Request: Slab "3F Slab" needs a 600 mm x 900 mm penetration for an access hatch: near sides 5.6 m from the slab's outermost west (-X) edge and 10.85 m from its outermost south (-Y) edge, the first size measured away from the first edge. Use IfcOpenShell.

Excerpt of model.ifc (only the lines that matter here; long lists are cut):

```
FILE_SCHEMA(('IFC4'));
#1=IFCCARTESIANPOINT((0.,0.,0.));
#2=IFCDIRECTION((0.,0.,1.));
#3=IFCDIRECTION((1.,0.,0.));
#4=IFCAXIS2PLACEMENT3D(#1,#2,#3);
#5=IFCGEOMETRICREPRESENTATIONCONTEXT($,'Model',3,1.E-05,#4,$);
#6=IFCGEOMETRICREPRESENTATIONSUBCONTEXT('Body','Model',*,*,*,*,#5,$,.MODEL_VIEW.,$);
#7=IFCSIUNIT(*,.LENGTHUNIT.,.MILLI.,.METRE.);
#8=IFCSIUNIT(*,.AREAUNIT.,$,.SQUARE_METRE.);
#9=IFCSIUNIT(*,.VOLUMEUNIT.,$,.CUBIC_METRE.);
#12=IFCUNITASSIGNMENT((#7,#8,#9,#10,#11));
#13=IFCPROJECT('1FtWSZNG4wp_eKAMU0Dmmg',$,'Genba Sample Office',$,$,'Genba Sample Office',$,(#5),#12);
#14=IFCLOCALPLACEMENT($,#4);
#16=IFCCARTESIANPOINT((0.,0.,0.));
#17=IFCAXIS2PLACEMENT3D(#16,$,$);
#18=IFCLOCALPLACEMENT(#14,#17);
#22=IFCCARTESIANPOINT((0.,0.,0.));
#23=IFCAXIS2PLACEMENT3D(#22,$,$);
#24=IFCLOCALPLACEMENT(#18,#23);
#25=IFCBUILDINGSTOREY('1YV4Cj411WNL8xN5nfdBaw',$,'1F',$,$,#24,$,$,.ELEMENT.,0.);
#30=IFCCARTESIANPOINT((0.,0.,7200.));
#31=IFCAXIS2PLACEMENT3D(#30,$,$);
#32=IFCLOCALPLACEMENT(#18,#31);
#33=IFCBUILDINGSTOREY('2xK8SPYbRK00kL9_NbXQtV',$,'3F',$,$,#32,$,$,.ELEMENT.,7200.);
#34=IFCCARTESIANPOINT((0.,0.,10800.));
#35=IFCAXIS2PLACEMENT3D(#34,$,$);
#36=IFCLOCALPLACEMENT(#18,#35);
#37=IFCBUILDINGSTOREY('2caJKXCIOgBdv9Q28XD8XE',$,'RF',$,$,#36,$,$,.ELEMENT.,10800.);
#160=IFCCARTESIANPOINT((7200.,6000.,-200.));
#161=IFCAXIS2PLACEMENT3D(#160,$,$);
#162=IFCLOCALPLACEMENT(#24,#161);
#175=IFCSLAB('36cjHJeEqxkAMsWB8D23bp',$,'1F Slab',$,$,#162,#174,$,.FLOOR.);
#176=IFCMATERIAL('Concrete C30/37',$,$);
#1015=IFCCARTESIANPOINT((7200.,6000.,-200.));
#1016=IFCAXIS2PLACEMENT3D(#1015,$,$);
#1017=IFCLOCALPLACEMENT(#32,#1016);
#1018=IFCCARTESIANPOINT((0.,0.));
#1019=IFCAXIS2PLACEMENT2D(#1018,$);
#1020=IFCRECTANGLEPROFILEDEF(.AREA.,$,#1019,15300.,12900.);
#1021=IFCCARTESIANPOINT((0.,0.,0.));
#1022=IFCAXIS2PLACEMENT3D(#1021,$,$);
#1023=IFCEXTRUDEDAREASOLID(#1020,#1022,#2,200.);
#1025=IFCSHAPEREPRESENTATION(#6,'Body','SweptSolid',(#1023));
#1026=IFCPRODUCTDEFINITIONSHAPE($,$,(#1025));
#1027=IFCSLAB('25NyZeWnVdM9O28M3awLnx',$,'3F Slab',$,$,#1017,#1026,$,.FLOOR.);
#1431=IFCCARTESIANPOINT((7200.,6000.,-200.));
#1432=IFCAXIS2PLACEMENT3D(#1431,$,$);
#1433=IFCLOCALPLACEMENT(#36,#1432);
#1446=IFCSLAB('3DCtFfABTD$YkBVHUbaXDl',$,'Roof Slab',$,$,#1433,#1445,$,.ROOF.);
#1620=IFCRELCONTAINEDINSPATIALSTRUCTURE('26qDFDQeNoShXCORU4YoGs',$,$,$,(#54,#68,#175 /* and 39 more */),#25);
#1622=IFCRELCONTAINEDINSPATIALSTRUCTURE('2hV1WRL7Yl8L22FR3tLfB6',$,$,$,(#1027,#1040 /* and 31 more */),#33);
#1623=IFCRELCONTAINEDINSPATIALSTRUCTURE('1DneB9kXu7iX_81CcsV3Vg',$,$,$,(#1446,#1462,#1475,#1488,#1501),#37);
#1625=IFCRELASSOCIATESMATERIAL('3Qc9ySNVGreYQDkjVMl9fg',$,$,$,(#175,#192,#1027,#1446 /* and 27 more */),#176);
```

```python
import numpy as np
import ifcopenshell
import ifcopenshell.api.feature
import ifcopenshell.api.geometry
import ifcopenshell.api.root
import ifcopenshell.geom
import ifcopenshell.util.placement
import ifcopenshell.util.representation
import ifcopenshell.util.shape
import ifcopenshell.util.unit

model = ifcopenshell.open("model.ifc")
unit_scale = ifcopenshell.util.unit.calculate_unit_scale(model)
settings = ifcopenshell.geom.settings()


def volume(element):
    """Net volume in cubic metres, openings subtracted."""
    shape = ifcopenshell.geom.create_shape(settings, element)
    return ifcopenshell.util.shape.get_volume(shape.geometry)


slab = model.by_id(1027)
before = volume(slab)

# Extent in the slab's own axes, in metres. The edges named are its -X and -Y sides.
slab_shape = ifcopenshell.geom.create_shape(settings, slab)
vertices = ifcopenshell.util.shape.get_vertices(slab_shape.geometry)
x_min, y_min, bottom = vertices.min(axis=0)
top = vertices[:, 2].max()

opening = ifcopenshell.api.root.create_entity(model, ifc_class="IfcOpeningElement", name="Access hatch opening", predefined_type="OPENING")
context = ifcopenshell.util.representation.get_context(model, "Model", "Body", "MODEL_VIEW")
width, depth = 0.6, 0.9
outline = [(0.0, 0.0), (width, 0.0), (width, depth), (0.0, depth), (0.0, 0.0)]
# Overshoot both faces by 50 mm so the cut is clean.
shape = ifcopenshell.api.geometry.add_slab_representation(
    model, context=context, depth=top - bottom + 0.1, polyline=outline
)
ifcopenshell.api.geometry.assign_representation(model, product=opening, representation=shape)

matrix = ifcopenshell.util.placement.get_local_placement(slab.ObjectPlacement)
matrix[:, 3] = matrix @ np.append(np.array([x_min + 5.6, y_min + 10.85, bottom - 0.05]) / unit_scale, 1.0)
ifcopenshell.api.geometry.edit_object_placement(model, product=opening, matrix=matrix, is_si=False)
ifcopenshell.api.feature.add_feature(model, feature=opening, element=slab)

after = volume(slab)

print(f"slab volume {before:.3f} -> {after:.3f} m3")

model.write("model_rev.ifc")
```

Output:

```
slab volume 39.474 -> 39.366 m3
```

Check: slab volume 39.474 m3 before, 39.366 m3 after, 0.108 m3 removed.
